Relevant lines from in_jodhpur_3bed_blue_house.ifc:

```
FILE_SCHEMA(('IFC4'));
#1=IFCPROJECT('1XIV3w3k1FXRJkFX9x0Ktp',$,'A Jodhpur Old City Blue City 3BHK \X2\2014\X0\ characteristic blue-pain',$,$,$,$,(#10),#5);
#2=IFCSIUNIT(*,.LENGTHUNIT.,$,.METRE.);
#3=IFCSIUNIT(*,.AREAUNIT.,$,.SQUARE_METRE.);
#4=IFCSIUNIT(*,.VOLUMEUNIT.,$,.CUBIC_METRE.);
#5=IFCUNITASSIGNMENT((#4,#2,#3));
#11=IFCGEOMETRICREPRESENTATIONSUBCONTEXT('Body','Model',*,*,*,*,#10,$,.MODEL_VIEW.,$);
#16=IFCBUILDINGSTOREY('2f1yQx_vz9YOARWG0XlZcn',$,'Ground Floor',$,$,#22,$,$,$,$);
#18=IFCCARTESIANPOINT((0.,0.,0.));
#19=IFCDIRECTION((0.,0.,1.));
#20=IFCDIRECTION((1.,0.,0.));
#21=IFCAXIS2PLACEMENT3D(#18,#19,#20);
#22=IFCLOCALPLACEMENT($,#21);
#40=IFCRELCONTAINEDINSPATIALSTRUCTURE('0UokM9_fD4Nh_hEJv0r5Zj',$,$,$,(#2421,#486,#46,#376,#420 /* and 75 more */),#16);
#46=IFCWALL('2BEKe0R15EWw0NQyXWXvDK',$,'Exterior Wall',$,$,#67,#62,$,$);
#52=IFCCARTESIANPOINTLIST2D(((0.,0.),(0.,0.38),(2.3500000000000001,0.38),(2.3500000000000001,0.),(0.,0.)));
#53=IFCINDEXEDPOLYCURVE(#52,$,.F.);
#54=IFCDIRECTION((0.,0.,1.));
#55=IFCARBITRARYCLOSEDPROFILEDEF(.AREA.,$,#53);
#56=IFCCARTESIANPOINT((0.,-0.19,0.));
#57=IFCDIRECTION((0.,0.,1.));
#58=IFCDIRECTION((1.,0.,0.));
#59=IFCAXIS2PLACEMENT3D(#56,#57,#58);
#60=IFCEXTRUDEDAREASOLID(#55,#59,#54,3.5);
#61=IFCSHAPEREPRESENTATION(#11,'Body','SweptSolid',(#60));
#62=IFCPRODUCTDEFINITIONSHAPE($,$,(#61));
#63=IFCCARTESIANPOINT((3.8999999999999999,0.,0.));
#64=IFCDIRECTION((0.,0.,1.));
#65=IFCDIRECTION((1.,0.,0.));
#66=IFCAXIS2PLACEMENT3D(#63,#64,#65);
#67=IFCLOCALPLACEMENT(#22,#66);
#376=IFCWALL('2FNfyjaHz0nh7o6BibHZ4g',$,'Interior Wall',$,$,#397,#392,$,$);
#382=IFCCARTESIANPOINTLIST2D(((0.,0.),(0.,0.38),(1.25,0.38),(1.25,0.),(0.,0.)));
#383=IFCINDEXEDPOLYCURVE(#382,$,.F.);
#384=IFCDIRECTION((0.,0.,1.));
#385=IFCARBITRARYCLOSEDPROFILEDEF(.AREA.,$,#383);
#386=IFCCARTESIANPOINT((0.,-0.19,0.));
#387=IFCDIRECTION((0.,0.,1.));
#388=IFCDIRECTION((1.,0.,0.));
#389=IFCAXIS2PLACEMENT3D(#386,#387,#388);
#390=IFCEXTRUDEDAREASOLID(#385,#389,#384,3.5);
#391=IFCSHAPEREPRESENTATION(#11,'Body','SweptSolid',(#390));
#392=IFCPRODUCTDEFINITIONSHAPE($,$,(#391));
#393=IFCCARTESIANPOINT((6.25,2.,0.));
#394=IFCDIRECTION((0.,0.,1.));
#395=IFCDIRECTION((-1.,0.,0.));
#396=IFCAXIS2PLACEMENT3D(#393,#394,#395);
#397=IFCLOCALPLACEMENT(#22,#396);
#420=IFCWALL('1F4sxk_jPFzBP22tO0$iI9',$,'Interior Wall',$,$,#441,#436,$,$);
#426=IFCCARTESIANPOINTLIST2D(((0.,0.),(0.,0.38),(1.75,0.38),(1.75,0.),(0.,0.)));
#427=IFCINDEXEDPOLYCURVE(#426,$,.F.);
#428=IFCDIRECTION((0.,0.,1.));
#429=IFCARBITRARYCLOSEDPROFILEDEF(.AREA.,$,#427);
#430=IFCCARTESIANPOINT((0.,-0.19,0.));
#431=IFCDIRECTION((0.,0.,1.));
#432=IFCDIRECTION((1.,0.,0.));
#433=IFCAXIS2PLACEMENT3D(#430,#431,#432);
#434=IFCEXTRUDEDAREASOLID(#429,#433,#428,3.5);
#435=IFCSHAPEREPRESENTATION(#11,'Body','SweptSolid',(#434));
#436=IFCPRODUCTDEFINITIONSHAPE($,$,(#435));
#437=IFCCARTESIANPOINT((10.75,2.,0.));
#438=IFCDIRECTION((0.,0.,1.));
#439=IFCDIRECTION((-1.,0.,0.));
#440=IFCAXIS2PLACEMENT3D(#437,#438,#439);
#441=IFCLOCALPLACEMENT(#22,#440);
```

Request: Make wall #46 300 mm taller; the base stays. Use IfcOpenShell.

```python
import ifcopenshell
import ifcopenshell.geom
import ifcopenshell.util.representation
import ifcopenshell.util.shape
import ifcopenshell.util.unit

model = ifcopenshell.open("in_jodhpur_3bed_blue_house.ifc")
unit_scale = ifcopenshell.util.unit.calculate_unit_scale(model)
settings = ifcopenshell.geom.settings()


def volume(element):
    """Net volume in cubic metres, openings subtracted."""
    shape = ifcopenshell.geom.create_shape(settings, element)
    return ifcopenshell.util.shape.get_volume(shape.geometry)


wall = model.by_guid("2BEKe0R15EWw0NQyXWXvDK")
before = volume(wall)

body = ifcopenshell.util.representation.get_representation(wall, "Model", "Body")
solid = body.Items[0]
old_height = solid.Depth
solid.Depth += 0.3 / unit_scale
after = volume(wall)

print(f"height {old_height:g} -> {solid.Depth:g}, volume {before:.3f} -> {after:.3f} m3")

model.write("in_jodhpur_3bed_blue_house_edited.ifc")
```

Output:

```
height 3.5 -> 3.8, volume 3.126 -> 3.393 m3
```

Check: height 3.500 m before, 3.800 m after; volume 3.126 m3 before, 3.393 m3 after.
